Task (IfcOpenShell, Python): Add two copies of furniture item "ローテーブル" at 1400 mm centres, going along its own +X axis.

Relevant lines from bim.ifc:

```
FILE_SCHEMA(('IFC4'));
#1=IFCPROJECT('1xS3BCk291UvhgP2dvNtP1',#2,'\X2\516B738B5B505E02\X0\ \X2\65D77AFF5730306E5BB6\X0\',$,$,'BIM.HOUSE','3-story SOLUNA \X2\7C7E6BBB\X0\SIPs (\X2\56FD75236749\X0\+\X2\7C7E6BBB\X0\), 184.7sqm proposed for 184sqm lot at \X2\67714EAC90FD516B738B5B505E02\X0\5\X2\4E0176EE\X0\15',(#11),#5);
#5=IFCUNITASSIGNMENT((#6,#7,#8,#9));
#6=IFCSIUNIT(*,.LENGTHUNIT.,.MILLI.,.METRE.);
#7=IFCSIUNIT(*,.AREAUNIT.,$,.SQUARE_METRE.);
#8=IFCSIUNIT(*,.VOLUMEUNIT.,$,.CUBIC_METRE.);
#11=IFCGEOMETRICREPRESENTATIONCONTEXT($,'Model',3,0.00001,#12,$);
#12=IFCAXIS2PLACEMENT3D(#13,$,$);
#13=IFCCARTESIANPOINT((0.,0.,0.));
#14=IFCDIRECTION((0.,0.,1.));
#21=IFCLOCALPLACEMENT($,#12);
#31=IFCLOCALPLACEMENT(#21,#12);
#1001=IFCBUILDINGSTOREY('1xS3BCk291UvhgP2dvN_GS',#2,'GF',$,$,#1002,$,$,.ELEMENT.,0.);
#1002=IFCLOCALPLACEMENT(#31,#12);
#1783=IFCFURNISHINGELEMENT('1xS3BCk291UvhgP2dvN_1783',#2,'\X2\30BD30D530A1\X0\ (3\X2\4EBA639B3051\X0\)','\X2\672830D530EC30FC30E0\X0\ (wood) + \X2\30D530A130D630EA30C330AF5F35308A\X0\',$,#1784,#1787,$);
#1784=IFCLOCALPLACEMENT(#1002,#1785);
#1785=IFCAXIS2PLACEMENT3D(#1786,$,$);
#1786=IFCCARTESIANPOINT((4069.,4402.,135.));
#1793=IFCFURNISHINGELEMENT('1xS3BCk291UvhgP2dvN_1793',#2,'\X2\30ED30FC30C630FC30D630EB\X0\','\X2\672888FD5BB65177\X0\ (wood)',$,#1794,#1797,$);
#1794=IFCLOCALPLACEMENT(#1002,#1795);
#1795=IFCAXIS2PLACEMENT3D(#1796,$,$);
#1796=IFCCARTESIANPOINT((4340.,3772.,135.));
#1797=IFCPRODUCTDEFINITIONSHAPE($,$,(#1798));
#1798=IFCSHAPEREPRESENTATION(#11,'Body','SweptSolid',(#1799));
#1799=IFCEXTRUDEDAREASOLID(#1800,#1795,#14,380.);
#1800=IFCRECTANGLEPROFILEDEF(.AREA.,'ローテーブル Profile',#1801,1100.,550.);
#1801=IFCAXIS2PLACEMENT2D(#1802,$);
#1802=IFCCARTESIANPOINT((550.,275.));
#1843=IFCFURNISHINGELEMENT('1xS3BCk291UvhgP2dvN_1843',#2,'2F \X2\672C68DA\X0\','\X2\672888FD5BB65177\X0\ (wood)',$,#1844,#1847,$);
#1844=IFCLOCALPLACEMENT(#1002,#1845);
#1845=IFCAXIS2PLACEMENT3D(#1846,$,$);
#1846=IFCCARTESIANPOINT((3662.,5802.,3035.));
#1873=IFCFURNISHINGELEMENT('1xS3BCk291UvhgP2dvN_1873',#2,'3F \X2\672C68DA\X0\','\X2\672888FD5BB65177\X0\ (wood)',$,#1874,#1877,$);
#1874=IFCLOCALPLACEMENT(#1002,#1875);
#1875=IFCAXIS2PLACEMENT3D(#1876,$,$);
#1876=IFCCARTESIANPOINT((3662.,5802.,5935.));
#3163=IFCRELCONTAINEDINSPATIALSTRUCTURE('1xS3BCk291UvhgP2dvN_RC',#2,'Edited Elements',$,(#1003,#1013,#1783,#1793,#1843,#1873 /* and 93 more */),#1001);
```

```python
import ifcopenshell
import ifcopenshell.api.geometry
import ifcopenshell.api.root
import ifcopenshell.util.element
import ifcopenshell.util.placement
import ifcopenshell.util.unit

model = ifcopenshell.open("bim.ifc")
unit_scale = ifcopenshell.util.unit.calculate_unit_scale(model)


def reuse_history(source, copy):
    """copy_class also copies each property set's owner history, people and application; keep the originals."""
    for rel in copy.IsDefinedBy:
        if rel.is_a("IfcRelDefinesByProperties") and (history := rel.RelatingPropertyDefinition.OwnerHistory):
            rel.RelatingPropertyDefinition.OwnerHistory = source.OwnerHistory
            ifcopenshell.util.element.remove_deep2(model, history)


source = model.by_guid("1xS3BCk291UvhgP2dvN_1793")
base = ifcopenshell.util.placement.get_local_placement(source.ObjectPlacement)
step = base[:3, 0] * 1.4 / unit_scale

for i in range(1, 3):
    copy = ifcopenshell.api.root.copy_class(model, product=source)
    copy.Representation = ifcopenshell.util.element.copy_deep(
        model, source.Representation, exclude=["IfcGeometricRepresentationContext", "IfcRepresentationMap"]
    )
    reuse_history(source, copy)
    matrix = base.copy()
    matrix[:3, 3] += i * step
    print("added at", matrix[:3, 3].round(3) + 0.0)
    ifcopenshell.api.geometry.edit_object_placement(model, product=copy, matrix=matrix, is_si=False)

model.write("bim-out.ifc")
```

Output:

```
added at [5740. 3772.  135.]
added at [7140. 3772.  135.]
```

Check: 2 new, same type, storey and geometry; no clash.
